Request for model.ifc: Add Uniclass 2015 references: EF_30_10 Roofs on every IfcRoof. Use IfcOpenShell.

First a look at what the model holds.

```python
import ifcopenshell

model = ifcopenshell.open("model.ifc")
print(model.schema)
print("classifications:", [c.Name for c in model.by_type("IfcClassification")])
for ifc_class in ("IfcDoor", "IfcRoof", "IfcStair", "IfcWall", "IfcWindow"):
    print(ifc_class, len(model.by_type(ifc_class)))
```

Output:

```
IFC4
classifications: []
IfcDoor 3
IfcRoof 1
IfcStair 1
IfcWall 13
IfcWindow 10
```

```python
import ifcopenshell
import ifcopenshell.api.classification

model = ifcopenshell.open("model.ifc")

system = ifcopenshell.api.classification.add_classification(model, classification="Uniclass 2015")

codes = {
    "IfcRoof": ("EF_30_10", "Roofs"),
}
for ifc_class, (code, name) in codes.items():
    products = model.by_type(ifc_class)
    ifcopenshell.api.classification.add_reference(
        model, products=products, classification=system, identification=code, name=name
    )
    print(code, len(products))

model.write("model_edited.ifc")
```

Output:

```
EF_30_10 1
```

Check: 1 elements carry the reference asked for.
